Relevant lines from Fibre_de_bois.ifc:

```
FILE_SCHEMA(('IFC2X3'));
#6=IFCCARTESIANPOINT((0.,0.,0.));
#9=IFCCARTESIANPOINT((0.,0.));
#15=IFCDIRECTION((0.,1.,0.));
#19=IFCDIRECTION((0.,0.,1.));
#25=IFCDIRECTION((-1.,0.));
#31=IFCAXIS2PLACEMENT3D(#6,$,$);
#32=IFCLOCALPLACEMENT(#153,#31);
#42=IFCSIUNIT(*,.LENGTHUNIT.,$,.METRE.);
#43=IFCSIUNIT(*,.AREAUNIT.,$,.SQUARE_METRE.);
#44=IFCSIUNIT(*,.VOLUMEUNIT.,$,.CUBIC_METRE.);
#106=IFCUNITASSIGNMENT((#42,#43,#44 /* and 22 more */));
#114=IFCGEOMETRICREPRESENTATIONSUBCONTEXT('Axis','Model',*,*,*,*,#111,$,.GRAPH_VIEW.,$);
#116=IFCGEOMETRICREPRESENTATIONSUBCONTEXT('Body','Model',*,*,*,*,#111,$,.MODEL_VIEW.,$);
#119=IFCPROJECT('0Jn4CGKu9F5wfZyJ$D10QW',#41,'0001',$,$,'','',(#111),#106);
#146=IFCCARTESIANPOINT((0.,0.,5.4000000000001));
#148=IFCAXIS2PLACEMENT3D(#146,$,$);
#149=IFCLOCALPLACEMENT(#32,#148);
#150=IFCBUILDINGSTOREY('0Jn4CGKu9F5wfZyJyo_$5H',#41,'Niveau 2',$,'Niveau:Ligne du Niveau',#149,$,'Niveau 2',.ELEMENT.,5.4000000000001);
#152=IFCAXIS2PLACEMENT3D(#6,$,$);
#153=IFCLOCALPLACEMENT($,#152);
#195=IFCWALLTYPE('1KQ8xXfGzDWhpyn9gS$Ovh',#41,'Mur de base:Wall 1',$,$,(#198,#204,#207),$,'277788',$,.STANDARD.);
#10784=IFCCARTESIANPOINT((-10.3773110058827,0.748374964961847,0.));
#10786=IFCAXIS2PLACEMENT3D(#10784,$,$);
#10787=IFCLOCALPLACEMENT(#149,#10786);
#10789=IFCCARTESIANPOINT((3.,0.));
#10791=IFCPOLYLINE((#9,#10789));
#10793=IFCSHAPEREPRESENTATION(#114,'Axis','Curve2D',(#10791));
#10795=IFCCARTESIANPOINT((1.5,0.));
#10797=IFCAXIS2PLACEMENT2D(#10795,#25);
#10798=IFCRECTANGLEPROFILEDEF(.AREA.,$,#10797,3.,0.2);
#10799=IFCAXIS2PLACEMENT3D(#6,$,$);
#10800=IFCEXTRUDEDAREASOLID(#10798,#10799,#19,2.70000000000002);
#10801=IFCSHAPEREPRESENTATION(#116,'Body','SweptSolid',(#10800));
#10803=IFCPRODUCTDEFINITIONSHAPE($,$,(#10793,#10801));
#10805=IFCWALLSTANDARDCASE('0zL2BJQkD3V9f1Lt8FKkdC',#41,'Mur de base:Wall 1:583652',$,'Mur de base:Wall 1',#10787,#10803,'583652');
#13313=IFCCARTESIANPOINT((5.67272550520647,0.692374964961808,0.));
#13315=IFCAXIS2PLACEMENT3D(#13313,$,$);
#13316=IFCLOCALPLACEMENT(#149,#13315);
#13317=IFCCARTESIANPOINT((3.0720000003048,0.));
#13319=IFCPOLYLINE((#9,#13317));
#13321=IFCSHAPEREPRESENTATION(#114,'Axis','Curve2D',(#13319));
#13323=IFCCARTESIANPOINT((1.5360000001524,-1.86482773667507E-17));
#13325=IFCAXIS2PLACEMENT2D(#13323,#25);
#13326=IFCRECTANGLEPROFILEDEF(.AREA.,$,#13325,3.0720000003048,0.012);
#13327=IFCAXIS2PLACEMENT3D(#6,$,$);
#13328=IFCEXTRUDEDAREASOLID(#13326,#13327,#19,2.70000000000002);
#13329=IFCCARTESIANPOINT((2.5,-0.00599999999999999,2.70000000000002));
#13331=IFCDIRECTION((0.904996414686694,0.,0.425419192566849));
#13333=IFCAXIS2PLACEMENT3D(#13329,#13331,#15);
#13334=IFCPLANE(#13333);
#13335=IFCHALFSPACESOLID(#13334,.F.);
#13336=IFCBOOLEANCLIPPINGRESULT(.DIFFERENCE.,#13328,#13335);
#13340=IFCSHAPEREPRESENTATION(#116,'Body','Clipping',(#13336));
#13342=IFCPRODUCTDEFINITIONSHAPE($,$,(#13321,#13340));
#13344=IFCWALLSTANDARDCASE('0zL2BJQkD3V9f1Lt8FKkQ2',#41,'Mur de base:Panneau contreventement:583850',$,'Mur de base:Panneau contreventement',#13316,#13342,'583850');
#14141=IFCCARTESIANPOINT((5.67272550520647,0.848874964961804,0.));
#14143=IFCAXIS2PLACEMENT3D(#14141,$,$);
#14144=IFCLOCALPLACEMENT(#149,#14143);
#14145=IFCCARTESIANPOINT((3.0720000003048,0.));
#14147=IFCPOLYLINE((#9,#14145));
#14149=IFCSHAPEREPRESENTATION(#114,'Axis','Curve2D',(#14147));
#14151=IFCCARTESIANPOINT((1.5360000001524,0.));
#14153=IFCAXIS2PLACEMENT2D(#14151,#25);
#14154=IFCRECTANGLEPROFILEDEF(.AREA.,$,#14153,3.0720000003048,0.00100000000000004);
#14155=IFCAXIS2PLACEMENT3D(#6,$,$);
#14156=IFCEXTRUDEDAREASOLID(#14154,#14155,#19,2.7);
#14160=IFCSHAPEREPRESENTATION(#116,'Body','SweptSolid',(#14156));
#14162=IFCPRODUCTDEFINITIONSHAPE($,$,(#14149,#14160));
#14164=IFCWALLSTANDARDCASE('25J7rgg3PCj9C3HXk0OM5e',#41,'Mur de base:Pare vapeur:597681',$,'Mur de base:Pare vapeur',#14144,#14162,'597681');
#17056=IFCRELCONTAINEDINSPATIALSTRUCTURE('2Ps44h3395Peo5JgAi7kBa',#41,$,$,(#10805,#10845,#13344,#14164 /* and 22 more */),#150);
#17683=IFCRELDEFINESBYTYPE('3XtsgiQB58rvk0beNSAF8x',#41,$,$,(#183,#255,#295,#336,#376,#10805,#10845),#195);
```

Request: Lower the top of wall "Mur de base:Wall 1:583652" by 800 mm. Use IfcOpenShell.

```python
import ifcopenshell
import ifcopenshell.geom
import ifcopenshell.util.representation
import ifcopenshell.util.shape
import ifcopenshell.util.unit

model = ifcopenshell.open("Fibre_de_bois.ifc")
unit_scale = ifcopenshell.util.unit.calculate_unit_scale(model)
settings = ifcopenshell.geom.settings()


def volume(element):
    """Net volume in cubic metres, openings subtracted."""
    shape = ifcopenshell.geom.create_shape(settings, element)
    return ifcopenshell.util.shape.get_volume(shape.geometry)


wall = model.by_guid("0zL2BJQkD3V9f1Lt8FKkdC")
before = volume(wall)

body = ifcopenshell.util.representation.get_representation(wall, "Model", "Body")
solid = body.Items[0]
old_height = solid.Depth
solid.Depth -= 0.8 / unit_scale
after = volume(wall)

print(f"height {old_height:g} -> {solid.Depth:g}, volume {before:.3f} -> {after:.3f} m3")

model.write("Fibre_de_bois_v2.ifc")
```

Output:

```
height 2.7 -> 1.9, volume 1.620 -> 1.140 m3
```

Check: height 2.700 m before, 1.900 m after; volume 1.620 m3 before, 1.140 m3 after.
